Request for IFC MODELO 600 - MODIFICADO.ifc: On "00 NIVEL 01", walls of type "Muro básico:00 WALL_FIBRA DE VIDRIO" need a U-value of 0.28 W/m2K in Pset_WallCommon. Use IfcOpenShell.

First a look at what the model holds.

```python
import ifcopenshell
import ifcopenshell.util.element

model = ifcopenshell.open("IFC MODELO 600 - MODIFICADO.ifc")
print(model.schema)
storey = next(s for s in model.by_type("IfcBuildingStorey") if s.Name == "00 NIVEL 01")
walls = [e for e in ifcopenshell.util.element.get_decomposition(storey) if e.is_a("IfcWall")]
seen = {}
for e in walls:
    element_type = ifcopenshell.util.element.get_type(e)
    key = (element_type.Name if element_type != e and element_type else None, ifcopenshell.util.element.get_pset(e, "Pset_WallCommon", "ThermalTransmittance"))
    seen[key] = seen.get(key, 0) + 1
for (name, value), count in sorted(seen.items(), key=str):
    print(count, "x", name, "|", value)
```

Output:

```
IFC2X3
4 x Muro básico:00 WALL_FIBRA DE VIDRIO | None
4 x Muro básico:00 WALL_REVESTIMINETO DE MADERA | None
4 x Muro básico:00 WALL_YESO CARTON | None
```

```python
import ifcopenshell
import ifcopenshell.api.pset
import ifcopenshell.util.element

model = ifcopenshell.open("IFC MODELO 600 - MODIFICADO.ifc")

storey = next(s for s in model.by_type("IfcBuildingStorey") if s.Name == "00 NIVEL 01")
walls = [e for e in ifcopenshell.util.element.get_decomposition(storey) if e.is_a("IfcWall")]

count = 0
for e in walls:
    element_type = ifcopenshell.util.element.get_type(e)
    if element_type in (None, e) or element_type.Name != "Muro básico:00 WALL_FIBRA DE VIDRIO":
        continue
    # add_pset returns the element's existing set when there is one.
    pset = ifcopenshell.api.pset.add_pset(model, product=e, name="Pset_WallCommon")
    ifcopenshell.api.pset.edit_pset(model, pset=pset, properties={"ThermalTransmittance": 0.28})
    count += 1

print(count, "walls updated")

model.write("IFC MODELO 600 - MODIFICADO_edited.ifc")
```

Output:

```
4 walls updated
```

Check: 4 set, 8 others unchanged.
